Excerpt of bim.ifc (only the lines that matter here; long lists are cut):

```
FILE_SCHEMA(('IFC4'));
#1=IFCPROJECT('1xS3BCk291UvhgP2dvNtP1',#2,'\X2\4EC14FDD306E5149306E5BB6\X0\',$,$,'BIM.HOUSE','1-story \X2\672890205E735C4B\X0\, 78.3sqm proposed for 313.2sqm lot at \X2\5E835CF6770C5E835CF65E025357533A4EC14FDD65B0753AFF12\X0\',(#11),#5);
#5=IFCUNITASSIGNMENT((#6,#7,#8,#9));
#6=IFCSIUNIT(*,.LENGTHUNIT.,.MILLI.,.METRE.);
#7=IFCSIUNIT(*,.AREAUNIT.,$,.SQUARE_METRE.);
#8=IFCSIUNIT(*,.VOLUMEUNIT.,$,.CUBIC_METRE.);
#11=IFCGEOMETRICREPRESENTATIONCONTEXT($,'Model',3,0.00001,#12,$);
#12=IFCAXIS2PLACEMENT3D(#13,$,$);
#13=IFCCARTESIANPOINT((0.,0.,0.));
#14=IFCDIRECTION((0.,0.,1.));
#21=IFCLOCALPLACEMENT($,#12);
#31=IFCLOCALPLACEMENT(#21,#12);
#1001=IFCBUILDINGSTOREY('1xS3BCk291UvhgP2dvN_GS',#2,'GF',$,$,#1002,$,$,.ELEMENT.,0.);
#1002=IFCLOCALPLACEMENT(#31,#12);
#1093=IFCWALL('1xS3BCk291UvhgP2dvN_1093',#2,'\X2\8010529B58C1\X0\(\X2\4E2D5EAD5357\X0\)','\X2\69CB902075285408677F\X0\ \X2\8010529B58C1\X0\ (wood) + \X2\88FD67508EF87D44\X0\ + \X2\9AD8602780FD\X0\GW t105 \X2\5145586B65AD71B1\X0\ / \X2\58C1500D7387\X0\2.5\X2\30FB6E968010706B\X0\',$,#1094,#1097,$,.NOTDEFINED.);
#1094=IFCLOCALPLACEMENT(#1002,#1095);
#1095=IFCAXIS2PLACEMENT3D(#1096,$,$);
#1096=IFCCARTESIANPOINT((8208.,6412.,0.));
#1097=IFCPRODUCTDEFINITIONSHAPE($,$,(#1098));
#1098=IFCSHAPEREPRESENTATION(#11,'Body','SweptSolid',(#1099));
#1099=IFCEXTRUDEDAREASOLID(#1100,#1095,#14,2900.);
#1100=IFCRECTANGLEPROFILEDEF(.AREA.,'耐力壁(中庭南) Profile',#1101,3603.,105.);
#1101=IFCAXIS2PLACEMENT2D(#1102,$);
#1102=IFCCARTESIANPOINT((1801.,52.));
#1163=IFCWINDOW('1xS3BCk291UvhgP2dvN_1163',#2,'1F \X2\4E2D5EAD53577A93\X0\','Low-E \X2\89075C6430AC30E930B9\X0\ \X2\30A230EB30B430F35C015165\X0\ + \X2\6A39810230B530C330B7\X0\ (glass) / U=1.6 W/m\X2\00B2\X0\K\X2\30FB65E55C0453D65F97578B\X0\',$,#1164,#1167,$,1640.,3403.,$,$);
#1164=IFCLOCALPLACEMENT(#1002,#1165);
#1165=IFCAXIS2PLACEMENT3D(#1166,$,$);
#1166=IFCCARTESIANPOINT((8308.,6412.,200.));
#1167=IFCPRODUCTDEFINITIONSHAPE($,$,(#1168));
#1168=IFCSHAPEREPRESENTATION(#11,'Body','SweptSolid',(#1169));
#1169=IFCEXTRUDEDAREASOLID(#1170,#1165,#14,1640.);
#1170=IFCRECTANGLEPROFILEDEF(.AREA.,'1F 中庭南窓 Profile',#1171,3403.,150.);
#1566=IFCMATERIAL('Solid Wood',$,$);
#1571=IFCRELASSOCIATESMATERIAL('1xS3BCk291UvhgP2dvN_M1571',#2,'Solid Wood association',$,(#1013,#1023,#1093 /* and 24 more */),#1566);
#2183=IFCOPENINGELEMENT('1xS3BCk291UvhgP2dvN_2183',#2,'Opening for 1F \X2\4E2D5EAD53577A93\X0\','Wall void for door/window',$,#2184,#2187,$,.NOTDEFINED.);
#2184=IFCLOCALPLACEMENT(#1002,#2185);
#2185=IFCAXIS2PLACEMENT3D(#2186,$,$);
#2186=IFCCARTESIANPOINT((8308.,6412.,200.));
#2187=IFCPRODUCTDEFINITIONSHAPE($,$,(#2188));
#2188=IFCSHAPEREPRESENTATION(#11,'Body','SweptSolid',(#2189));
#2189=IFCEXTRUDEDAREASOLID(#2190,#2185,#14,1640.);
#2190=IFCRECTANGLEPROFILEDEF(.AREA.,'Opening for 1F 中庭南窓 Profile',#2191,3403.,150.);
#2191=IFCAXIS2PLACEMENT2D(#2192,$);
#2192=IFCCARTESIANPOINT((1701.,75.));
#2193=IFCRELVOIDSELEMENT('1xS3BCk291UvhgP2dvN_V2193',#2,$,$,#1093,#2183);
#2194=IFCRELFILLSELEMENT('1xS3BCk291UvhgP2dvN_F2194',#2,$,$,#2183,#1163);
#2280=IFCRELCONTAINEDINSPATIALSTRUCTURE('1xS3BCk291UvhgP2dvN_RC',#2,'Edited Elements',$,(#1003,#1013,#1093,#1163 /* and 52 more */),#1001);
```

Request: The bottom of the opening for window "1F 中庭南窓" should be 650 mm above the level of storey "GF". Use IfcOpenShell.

```python
import numpy as np
import ifcopenshell
import ifcopenshell.api.geometry
import ifcopenshell.geom
import ifcopenshell.util.element
import ifcopenshell.util.placement
import ifcopenshell.util.shape
import ifcopenshell.util.unit

model = ifcopenshell.open("bim.ifc")
unit_scale = ifcopenshell.util.unit.calculate_unit_scale(model)

window = model.by_guid("1xS3BCk291UvhgP2dvN_1163")
opening = window.FillsVoids[0].RelatingOpeningElement
storey = ifcopenshell.util.element.get_container(window, ifc_class="IfcBuildingStorey")
level = ifcopenshell.util.placement.get_local_placement(storey.ObjectPlacement)[2, 3]

# The opening's origin need not be at the sill, so measure its lowest point.
shape = ifcopenshell.geom.create_shape(ifcopenshell.geom.settings(), opening)
bottom = ifcopenshell.util.shape.get_shape_bottom_elevation(shape, shape.geometry) / unit_scale
dz = level + 650.0 - bottom

shift = np.array([0.0, 0.0, dz])
# The window is not placed relative to its opening, so move both.
for product in (opening, window):
    matrix = ifcopenshell.util.placement.get_local_placement(product.ObjectPlacement)
    matrix[:3, 3] += shift
    ifcopenshell.api.geometry.edit_object_placement(model, product=product, matrix=matrix, is_si=False)

print(f"moved by {dz * unit_scale:+.3f} m")

model.write("bim-out.ifc")
```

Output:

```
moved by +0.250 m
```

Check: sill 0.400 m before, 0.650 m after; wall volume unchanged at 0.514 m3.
